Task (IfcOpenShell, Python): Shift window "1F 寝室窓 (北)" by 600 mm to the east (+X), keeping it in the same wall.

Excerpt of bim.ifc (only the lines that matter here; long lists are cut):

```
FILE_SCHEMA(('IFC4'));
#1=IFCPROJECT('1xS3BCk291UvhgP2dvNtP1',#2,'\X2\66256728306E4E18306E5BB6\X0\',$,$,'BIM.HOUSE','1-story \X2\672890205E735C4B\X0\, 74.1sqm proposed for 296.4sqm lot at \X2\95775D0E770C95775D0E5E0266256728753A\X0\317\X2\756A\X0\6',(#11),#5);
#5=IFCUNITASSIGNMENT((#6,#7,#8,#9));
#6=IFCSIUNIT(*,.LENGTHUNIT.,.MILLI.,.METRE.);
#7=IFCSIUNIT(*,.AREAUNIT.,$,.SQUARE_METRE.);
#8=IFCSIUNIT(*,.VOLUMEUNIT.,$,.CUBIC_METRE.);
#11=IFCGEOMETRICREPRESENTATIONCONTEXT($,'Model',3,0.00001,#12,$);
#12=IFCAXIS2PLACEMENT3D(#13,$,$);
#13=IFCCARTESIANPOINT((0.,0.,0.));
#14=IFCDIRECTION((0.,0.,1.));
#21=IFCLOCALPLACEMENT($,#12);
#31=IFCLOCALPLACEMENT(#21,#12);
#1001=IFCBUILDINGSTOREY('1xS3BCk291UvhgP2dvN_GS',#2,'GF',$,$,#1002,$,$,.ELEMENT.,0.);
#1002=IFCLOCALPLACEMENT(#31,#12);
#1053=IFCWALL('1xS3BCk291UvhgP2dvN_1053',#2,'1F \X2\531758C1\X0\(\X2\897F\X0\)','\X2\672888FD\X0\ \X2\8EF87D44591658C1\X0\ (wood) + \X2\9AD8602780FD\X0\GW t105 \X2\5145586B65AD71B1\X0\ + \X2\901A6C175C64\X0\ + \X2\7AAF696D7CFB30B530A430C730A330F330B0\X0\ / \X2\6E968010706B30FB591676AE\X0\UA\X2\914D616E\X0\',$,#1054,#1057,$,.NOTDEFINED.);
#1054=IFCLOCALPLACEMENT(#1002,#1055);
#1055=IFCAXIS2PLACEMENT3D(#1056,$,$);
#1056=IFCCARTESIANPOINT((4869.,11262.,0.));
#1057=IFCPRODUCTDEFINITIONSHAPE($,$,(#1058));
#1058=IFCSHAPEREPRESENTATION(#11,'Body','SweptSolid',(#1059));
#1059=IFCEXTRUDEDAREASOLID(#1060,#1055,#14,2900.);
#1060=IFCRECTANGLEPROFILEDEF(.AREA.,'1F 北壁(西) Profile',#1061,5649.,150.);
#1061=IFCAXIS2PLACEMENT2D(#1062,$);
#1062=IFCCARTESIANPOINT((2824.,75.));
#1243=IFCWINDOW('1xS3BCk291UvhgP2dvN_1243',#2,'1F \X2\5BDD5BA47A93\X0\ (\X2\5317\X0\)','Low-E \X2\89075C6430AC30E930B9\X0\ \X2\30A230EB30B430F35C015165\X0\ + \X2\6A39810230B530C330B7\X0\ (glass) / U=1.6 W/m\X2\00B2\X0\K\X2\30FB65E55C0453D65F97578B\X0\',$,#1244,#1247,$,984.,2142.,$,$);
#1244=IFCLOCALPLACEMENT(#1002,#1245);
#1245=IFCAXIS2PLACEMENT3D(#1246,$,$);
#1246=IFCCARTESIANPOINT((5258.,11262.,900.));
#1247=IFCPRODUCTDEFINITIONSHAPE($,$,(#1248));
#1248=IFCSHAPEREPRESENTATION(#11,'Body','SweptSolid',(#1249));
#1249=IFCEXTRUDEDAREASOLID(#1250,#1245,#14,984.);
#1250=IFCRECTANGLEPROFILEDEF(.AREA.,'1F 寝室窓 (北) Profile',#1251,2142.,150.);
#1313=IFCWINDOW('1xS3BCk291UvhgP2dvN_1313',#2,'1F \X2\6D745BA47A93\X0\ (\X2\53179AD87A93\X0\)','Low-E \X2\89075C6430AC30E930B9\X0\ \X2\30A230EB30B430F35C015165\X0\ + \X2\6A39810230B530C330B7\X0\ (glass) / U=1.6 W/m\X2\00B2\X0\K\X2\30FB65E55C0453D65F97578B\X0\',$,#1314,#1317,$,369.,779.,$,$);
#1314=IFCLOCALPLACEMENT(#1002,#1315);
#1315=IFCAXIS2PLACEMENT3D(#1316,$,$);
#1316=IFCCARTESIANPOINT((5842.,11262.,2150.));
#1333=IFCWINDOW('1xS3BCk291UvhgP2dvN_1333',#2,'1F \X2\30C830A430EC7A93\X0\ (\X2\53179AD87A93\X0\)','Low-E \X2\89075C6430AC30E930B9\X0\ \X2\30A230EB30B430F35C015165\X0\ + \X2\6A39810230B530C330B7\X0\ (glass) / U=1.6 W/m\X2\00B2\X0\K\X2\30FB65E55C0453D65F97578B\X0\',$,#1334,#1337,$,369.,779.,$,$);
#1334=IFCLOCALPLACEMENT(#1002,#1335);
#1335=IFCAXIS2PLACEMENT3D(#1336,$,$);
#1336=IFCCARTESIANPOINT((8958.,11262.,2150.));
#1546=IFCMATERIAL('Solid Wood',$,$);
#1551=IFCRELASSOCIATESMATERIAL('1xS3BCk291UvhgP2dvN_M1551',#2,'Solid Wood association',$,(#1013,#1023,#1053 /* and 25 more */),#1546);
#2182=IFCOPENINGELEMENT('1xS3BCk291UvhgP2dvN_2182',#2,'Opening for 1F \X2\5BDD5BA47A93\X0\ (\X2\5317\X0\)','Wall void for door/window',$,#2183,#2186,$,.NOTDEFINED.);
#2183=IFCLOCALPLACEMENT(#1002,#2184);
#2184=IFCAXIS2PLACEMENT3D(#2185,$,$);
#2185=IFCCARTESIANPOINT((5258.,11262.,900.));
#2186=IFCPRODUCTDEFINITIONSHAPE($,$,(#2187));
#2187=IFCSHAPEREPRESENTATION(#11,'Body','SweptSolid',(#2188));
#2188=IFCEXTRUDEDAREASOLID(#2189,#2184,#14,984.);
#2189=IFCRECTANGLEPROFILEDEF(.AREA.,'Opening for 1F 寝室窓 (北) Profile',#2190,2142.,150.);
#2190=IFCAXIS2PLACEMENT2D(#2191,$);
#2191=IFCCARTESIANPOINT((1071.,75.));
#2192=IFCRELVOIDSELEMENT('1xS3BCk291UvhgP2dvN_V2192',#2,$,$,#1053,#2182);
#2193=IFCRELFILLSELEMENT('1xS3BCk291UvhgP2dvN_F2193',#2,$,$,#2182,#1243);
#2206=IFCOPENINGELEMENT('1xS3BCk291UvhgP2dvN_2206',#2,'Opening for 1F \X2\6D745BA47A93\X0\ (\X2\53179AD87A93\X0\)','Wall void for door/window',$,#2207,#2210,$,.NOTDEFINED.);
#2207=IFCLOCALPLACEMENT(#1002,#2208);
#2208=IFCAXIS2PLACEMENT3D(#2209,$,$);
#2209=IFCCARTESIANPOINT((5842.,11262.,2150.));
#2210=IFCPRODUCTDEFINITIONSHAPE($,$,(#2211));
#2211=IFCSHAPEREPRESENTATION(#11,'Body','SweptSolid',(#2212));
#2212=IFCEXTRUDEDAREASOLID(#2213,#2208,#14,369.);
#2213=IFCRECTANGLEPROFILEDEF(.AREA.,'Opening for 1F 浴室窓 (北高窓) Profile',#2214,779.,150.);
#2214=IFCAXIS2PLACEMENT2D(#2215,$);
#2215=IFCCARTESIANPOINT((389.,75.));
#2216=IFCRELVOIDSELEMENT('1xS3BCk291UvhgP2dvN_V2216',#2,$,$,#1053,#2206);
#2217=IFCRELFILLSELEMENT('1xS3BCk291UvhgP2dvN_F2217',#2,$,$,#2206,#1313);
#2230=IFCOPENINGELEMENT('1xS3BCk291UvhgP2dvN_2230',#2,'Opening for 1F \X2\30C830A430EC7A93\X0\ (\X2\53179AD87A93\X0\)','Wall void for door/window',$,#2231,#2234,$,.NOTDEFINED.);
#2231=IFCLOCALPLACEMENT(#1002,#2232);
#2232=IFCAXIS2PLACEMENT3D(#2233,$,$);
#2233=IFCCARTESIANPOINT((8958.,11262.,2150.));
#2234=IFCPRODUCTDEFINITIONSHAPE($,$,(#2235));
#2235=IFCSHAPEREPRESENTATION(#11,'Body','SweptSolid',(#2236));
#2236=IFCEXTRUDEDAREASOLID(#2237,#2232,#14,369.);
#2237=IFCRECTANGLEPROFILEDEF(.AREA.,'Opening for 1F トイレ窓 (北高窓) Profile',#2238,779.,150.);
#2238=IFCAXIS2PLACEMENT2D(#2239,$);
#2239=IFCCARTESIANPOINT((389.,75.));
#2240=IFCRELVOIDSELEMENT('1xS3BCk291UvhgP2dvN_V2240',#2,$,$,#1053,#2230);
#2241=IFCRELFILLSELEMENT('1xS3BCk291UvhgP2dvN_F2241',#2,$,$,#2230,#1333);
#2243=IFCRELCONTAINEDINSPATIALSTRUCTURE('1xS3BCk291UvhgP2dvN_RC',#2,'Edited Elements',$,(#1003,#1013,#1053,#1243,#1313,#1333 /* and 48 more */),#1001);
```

```python
import ifcopenshell
import ifcopenshell.api.geometry
import ifcopenshell.util.placement
import ifcopenshell.util.unit

model = ifcopenshell.open("bim.ifc")
unit_scale = ifcopenshell.util.unit.calculate_unit_scale(model)

window = model.by_guid("1xS3BCk291UvhgP2dvN_1243")
opening = window.FillsVoids[0].RelatingOpeningElement
wall = opening.VoidsElements[0].RelatingBuildingElement

wall_matrix = ifcopenshell.util.placement.get_local_placement(wall.ObjectPlacement)
shift = wall_matrix[:3, 0] * 0.6 / unit_scale
before = ifcopenshell.util.placement.get_local_placement(window.ObjectPlacement)[:3, 3].copy()

# The window is not placed relative to its opening, so move both.
for product in (opening, window):
    matrix = ifcopenshell.util.placement.get_local_placement(product.ObjectPlacement)
    matrix[:3, 3] += shift
    ifcopenshell.api.geometry.edit_object_placement(model, product=product, matrix=matrix, is_si=False)

after = ifcopenshell.util.placement.get_local_placement(window.ObjectPlacement)[:3, 3]
print("window moved by", (after - before).round(3) + 0.0)

model.write("bim-out.ifc")
```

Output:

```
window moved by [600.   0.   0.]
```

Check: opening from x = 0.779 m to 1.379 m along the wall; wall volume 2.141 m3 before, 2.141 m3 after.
